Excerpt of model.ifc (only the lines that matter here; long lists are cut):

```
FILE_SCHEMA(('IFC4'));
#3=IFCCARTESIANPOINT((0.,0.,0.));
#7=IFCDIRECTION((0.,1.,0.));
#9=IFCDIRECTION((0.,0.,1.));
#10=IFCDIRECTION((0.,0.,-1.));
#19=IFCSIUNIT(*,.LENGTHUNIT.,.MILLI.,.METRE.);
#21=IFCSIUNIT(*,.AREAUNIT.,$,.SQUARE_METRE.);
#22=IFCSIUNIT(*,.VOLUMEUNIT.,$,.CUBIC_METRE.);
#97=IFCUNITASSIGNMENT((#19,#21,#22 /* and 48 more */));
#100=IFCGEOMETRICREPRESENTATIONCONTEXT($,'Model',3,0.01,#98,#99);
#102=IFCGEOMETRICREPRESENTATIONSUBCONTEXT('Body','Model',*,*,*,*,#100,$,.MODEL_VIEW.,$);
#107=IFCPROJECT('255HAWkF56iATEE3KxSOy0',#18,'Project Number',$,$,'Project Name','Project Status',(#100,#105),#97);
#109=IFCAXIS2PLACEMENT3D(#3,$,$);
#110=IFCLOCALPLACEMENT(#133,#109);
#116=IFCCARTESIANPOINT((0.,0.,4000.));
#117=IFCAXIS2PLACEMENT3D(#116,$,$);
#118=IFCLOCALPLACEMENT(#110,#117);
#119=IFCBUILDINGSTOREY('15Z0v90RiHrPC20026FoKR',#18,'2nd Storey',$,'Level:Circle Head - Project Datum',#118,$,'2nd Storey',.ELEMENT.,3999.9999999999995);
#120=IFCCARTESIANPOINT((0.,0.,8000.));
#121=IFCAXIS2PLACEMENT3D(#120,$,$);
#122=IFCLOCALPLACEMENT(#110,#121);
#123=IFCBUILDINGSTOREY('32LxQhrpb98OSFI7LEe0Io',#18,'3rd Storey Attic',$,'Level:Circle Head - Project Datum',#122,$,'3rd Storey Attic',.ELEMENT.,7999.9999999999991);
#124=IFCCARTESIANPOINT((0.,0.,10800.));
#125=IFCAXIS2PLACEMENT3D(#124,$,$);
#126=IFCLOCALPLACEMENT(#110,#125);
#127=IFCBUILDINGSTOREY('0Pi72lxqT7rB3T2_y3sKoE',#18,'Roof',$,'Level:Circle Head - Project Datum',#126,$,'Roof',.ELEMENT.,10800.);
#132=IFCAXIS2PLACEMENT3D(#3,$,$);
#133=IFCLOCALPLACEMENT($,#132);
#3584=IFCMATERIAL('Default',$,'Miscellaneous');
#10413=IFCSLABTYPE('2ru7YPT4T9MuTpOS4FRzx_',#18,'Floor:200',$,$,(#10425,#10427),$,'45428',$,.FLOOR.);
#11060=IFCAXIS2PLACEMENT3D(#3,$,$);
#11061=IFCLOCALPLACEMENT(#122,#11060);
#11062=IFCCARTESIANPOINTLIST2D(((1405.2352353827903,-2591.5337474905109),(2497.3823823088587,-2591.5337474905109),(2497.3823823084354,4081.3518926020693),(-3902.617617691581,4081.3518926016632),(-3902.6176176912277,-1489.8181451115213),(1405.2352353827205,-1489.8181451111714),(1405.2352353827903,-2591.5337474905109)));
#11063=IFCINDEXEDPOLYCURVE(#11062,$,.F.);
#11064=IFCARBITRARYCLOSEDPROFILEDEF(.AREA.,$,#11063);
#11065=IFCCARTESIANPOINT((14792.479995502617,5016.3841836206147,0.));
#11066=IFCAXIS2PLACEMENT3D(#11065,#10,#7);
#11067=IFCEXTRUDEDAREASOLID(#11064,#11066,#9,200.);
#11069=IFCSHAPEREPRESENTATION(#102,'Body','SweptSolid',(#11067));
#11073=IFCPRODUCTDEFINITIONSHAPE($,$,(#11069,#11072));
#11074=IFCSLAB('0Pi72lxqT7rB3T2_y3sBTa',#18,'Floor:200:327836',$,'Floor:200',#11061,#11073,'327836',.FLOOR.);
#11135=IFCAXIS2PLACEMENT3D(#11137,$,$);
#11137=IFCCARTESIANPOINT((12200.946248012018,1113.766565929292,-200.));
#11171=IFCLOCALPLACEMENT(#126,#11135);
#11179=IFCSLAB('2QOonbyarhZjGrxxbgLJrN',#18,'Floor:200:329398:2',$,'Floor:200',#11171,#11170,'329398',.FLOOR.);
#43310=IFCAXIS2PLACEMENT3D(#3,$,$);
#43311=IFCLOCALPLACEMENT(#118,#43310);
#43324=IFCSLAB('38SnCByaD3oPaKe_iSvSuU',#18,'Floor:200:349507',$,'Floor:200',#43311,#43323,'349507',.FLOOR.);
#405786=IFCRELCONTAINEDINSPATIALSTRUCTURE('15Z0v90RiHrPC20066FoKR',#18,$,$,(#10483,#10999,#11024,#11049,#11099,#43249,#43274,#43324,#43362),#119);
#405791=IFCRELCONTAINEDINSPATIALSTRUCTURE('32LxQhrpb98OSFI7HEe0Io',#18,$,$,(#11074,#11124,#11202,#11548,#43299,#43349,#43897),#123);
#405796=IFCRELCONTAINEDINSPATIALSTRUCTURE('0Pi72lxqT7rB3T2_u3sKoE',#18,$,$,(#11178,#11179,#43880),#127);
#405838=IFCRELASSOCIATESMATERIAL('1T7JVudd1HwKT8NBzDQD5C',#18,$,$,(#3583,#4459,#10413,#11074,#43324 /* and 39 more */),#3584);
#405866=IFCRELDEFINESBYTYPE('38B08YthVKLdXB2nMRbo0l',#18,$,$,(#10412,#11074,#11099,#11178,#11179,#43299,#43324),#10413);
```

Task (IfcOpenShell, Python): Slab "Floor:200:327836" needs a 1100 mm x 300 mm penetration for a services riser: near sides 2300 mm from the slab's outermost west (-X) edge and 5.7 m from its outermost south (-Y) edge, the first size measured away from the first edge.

```python
import numpy as np
import ifcopenshell
import ifcopenshell.api.feature
import ifcopenshell.api.geometry
import ifcopenshell.api.root
import ifcopenshell.geom
import ifcopenshell.util.placement
import ifcopenshell.util.representation
import ifcopenshell.util.shape
import ifcopenshell.util.unit

model = ifcopenshell.open("model.ifc")
unit_scale = ifcopenshell.util.unit.calculate_unit_scale(model)
settings = ifcopenshell.geom.settings()


def volume(element):
    """Net volume in cubic metres, openings subtracted."""
    shape = ifcopenshell.geom.create_shape(settings, element)
    return ifcopenshell.util.shape.get_volume(shape.geometry)


slab = model.by_guid("0Pi72lxqT7rB3T2_y3sBTa")
before = volume(slab)

# Extent in the slab's own axes, in metres. The edges named are its -X and -Y sides.
slab_shape = ifcopenshell.geom.create_shape(settings, slab)
vertices = ifcopenshell.util.shape.get_vertices(slab_shape.geometry)
x_min, y_min, bottom = vertices.min(axis=0)
top = vertices[:, 2].max()

opening = ifcopenshell.api.root.create_entity(model, ifc_class="IfcOpeningElement", name="Services riser opening", predefined_type="OPENING")
context = ifcopenshell.util.representation.get_context(model, "Model", "Body", "MODEL_VIEW")
width, depth = 1.1, 0.3
outline = [(0.0, 0.0), (width, 0.0), (width, depth), (0.0, depth), (0.0, 0.0)]
# Overshoot both faces by 50 mm so the cut is clean.
shape = ifcopenshell.api.geometry.add_slab_representation(
    model, context=context, depth=top - bottom + 0.1, polyline=outline
)
ifcopenshell.api.geometry.assign_representation(model, product=opening, representation=shape)

matrix = ifcopenshell.util.placement.get_local_placement(slab.ObjectPlacement)
matrix[:, 3] = matrix @ np.append(np.array([x_min + 2.3, y_min + 5.7, bottom - 0.05]) / unit_scale, 1.0)
ifcopenshell.api.geometry.edit_object_placement(model, product=opening, matrix=matrix, is_si=False)
ifcopenshell.api.feature.add_feature(model, feature=opening, element=slab)

after = volume(slab)

print(f"slab volume {before:.3f} -> {after:.3f} m3")

model.write("model_updated.ifc")
```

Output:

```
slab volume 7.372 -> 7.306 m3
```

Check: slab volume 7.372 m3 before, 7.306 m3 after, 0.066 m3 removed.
